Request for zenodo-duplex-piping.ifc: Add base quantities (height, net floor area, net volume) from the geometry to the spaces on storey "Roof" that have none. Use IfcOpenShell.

First a look at what the model holds.

```python
import ifcopenshell
import ifcopenshell.util.element
import ifcopenshell.util.unit

model = ifcopenshell.open("zenodo-duplex-piping.ifc")
print(model.schema)
for unit_type in ("LENGTHUNIT", "AREAUNIT", "VOLUMEUNIT"):
    print(unit_type, ifcopenshell.util.unit.calculate_unit_scale(model, unit_type))
storey = next(s for s in model.by_type("IfcBuildingStorey") if s.Name == "Roof")
spaces = [e for e in ifcopenshell.util.element.get_decomposition(storey) if e.is_a("IfcSpace")]
for e in sorted(spaces, key=lambda e: e.id()):
    print(e.id(), e.is_a(), e.Name, list(ifcopenshell.util.element.get_psets(e, qtos_only=True)), sep=" | ")
```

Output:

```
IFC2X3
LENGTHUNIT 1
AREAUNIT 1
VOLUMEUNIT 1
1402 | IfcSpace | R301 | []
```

```python
import ifcopenshell
import ifcopenshell.api.pset
import ifcopenshell.geom
import ifcopenshell.util.element
import ifcopenshell.util.shape
import ifcopenshell.util.unit

model = ifcopenshell.open("zenodo-duplex-piping.ifc")
unit_scale = ifcopenshell.util.unit.calculate_unit_scale(model)
area_scale = ifcopenshell.util.unit.calculate_unit_scale(model, "AREAUNIT")
volume_scale = ifcopenshell.util.unit.calculate_unit_scale(model, "VOLUMEUNIT")
settings = ifcopenshell.geom.settings()

storey = next(s for s in model.by_type("IfcBuildingStorey") if s.Name == "Roof")
spaces = [e for e in ifcopenshell.util.element.get_decomposition(storey) if e.is_a("IfcSpace")]

for e in sorted(spaces, key=lambda e: e.id()):
    if ifcopenshell.util.element.get_psets(e, qtos_only=True, should_inherit=False):
        continue
    # Geometry comes back in metres, in the element's own axes.
    shape = ifcopenshell.geom.create_shape(settings, e)
    values = {
        "Height": ifcopenshell.util.shape.get_z(shape.geometry) / unit_scale,
        "NetFloorArea": ifcopenshell.util.shape.get_footprint_area(shape.geometry) / area_scale,
        "NetVolume": ifcopenshell.util.shape.get_volume(shape.geometry) / volume_scale,
    }
    qto = ifcopenshell.api.pset.add_qto(model, product=e, name="BaseQuantities")
    ifcopenshell.api.pset.edit_qto(model, qto=qto, properties=values)
    print(e.id(), {k: round(v, 3) for k, v in values.items()})

model.write("zenodo-duplex-piping_updated.ifc")
```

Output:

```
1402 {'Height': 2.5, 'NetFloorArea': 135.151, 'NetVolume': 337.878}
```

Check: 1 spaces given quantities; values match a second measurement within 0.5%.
